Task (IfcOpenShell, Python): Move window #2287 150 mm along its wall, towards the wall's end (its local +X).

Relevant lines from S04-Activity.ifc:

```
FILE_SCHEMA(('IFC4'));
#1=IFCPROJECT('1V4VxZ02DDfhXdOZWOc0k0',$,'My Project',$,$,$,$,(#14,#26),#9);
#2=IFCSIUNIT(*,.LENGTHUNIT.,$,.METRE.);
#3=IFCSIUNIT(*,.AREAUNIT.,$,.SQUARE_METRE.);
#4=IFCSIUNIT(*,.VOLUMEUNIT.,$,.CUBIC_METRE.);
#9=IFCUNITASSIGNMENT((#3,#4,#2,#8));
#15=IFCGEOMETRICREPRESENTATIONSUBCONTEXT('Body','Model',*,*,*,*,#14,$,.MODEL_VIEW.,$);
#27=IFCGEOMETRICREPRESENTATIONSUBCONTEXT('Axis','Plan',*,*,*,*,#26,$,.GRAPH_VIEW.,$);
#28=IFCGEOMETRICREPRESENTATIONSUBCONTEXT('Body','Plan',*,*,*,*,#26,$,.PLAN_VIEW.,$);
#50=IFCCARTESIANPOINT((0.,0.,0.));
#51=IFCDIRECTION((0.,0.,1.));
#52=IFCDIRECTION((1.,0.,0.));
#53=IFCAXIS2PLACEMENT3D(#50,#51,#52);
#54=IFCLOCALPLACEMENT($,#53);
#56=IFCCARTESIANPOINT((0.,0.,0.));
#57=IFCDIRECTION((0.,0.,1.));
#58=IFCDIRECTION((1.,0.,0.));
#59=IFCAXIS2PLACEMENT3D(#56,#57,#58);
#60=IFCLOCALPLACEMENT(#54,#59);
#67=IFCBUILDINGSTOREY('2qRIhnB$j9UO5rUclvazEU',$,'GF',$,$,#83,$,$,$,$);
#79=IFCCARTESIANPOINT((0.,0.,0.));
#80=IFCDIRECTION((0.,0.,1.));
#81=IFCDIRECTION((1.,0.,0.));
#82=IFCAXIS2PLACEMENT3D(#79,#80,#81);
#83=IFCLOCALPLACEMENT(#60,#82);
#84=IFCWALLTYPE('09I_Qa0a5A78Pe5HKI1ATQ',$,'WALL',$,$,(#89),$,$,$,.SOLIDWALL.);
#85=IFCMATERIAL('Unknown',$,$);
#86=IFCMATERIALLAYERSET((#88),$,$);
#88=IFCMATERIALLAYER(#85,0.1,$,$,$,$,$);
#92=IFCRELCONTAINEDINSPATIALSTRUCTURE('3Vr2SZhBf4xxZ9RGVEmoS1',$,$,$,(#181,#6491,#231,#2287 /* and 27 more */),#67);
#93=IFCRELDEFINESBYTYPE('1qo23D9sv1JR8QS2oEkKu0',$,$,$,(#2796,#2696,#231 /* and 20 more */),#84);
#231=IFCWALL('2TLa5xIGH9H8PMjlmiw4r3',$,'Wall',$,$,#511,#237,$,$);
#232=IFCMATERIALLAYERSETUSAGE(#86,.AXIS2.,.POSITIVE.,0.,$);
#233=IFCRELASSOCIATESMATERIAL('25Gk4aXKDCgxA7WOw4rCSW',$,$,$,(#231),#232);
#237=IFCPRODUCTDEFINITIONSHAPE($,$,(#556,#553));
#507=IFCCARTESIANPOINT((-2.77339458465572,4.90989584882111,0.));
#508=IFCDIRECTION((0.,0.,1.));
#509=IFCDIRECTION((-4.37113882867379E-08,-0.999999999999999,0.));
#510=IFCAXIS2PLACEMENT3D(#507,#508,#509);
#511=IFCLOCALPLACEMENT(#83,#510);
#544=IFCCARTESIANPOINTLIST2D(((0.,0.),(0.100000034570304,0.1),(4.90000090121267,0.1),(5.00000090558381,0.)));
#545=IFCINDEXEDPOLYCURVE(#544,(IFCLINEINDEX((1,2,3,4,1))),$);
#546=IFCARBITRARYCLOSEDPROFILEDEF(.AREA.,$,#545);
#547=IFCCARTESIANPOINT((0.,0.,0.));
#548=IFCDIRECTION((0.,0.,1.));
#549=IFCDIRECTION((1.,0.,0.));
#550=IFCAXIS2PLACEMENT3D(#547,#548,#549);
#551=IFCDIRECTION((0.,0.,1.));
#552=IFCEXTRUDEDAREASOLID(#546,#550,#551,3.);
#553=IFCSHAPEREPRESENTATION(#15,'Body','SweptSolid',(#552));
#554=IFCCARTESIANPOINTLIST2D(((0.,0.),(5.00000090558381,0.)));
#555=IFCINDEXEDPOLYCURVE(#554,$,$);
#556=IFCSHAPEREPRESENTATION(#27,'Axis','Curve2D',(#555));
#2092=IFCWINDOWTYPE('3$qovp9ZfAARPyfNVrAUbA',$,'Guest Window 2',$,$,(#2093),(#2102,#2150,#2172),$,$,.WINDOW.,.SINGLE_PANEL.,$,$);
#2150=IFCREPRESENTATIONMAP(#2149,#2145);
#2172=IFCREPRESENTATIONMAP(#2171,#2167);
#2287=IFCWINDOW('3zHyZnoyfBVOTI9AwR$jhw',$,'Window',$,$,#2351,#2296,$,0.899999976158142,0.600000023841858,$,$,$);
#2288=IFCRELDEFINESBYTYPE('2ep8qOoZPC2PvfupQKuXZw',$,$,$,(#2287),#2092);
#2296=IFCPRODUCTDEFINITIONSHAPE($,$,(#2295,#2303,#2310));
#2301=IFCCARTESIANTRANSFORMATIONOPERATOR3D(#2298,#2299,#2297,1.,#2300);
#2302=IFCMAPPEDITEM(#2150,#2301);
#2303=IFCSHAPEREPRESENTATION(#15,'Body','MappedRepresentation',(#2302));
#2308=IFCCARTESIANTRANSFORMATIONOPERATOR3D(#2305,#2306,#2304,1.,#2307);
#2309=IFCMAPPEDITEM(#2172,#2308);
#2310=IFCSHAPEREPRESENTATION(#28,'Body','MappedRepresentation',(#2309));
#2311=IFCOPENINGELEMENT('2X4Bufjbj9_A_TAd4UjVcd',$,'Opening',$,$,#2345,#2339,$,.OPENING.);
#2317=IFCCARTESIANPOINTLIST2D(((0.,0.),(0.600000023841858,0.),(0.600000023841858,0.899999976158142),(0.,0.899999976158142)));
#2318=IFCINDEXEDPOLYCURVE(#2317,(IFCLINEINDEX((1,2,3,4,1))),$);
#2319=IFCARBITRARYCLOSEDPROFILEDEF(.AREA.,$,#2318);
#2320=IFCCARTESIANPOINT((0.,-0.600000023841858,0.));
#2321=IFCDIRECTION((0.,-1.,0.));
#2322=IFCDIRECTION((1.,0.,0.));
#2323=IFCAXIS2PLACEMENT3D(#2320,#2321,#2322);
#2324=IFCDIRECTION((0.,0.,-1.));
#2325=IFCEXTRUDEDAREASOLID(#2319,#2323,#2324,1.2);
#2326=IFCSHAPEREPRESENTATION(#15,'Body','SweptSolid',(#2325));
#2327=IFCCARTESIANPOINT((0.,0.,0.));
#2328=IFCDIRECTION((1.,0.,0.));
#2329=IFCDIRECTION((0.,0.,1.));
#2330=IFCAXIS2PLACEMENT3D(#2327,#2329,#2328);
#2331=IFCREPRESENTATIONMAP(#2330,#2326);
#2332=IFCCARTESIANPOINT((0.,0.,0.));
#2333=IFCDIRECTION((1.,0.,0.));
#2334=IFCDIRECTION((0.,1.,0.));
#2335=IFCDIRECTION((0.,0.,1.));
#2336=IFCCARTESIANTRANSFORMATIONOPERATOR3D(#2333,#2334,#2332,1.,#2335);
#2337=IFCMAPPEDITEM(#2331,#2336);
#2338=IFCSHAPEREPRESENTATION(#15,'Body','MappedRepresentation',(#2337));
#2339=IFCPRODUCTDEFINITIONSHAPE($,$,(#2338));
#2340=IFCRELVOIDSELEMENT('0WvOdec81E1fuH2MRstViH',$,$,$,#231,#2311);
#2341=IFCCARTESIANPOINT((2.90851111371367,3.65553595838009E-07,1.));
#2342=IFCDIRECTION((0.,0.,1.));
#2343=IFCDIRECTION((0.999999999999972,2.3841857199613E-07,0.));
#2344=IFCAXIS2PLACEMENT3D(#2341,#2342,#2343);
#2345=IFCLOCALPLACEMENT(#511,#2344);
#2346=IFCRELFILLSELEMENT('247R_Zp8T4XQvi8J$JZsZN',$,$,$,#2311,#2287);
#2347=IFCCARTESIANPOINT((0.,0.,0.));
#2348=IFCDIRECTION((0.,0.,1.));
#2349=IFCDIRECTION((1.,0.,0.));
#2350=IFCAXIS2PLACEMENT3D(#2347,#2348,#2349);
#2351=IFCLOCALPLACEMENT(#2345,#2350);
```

```python
import ifcopenshell
import ifcopenshell.api.geometry
import ifcopenshell.util.placement

model = ifcopenshell.open("S04-Activity.ifc")

window = model.by_id(2287)
opening = window.FillsVoids[0].RelatingOpeningElement
wall = opening.VoidsElements[0].RelatingBuildingElement

wall_matrix = ifcopenshell.util.placement.get_local_placement(wall.ObjectPlacement)
shift = wall_matrix[:3, 0] * 0.15
before = ifcopenshell.util.placement.get_local_placement(window.ObjectPlacement)[:3, 3].copy()

# The window is placed relative to its opening, so it follows when the opening moves.
matrix = ifcopenshell.util.placement.get_local_placement(opening.ObjectPlacement)
matrix[:3, 3] += shift
ifcopenshell.api.geometry.edit_object_placement(
    model, product=opening, matrix=matrix, is_si=False, should_transform_children=True
)

after = ifcopenshell.util.placement.get_local_placement(window.ObjectPlacement)[:3, 3]
print("window moved by", (after - before).round(3) + 0.0)

model.write("S04-Activity_rev.ifc")
```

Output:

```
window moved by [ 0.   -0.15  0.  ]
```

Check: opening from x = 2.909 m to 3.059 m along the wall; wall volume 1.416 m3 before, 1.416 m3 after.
